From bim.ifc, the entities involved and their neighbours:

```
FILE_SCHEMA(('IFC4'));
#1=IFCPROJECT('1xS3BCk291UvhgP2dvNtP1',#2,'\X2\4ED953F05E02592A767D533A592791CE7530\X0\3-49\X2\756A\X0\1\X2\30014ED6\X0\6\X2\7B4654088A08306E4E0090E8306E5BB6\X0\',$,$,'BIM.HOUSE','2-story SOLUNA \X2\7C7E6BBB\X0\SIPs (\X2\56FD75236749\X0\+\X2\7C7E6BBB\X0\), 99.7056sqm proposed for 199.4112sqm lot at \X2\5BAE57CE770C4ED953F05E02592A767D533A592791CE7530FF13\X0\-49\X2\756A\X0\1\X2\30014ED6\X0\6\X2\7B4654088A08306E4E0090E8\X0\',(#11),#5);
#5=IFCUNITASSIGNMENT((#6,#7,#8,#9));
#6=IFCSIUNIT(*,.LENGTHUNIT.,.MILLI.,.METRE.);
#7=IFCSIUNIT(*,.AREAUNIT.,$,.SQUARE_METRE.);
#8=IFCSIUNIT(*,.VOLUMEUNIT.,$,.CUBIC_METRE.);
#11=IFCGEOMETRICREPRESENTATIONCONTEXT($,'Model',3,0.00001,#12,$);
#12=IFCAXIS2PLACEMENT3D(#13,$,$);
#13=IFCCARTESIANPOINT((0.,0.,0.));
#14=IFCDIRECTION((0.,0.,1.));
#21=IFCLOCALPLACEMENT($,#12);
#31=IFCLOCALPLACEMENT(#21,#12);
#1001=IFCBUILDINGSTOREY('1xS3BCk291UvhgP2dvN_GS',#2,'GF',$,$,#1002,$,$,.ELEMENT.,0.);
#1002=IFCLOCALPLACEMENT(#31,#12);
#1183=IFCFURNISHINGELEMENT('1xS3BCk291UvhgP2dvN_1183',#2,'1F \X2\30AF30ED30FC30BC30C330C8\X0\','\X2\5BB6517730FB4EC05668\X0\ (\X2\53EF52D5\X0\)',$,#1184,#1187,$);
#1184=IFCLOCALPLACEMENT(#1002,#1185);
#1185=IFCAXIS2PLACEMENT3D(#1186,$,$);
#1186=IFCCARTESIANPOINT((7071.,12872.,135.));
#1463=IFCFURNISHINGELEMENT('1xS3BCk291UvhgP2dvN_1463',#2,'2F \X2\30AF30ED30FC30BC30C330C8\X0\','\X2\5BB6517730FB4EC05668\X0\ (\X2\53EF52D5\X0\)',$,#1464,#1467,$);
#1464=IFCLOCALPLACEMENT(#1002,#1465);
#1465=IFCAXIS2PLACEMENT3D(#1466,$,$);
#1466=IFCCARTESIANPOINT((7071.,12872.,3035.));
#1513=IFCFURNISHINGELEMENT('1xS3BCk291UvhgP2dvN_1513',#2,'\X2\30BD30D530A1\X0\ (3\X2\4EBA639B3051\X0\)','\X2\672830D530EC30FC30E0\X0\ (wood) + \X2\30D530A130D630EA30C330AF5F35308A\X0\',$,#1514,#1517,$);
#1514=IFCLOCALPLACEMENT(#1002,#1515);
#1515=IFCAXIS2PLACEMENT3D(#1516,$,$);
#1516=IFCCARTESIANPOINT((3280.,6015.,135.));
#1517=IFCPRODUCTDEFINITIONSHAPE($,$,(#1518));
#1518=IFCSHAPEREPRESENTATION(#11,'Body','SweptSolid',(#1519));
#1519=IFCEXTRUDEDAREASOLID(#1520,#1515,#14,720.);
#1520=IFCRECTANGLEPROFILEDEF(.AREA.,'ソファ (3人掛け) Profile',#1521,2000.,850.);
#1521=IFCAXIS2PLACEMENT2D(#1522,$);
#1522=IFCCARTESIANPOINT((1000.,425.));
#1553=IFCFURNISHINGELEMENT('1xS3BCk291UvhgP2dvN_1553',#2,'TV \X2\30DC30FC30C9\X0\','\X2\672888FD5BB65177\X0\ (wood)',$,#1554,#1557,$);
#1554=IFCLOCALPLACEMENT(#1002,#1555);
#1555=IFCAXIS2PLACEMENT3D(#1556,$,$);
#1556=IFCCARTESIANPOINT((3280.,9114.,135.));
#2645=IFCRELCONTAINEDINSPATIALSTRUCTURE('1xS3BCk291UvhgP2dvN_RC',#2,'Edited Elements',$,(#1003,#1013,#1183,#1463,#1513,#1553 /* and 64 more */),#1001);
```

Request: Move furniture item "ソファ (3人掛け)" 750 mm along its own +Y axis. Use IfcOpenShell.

```python
import ifcopenshell
import ifcopenshell.api.geometry
import ifcopenshell.util.placement
import ifcopenshell.util.unit

model = ifcopenshell.open("bim.ifc")
unit_scale = ifcopenshell.util.unit.calculate_unit_scale(model)

item = model.by_guid("1xS3BCk291UvhgP2dvN_1513")
matrix = ifcopenshell.util.placement.get_local_placement(item.ObjectPlacement)
matrix[:3, 3] += matrix[:3, 1] * 0.75 / unit_scale
ifcopenshell.api.geometry.edit_object_placement(model, product=item, matrix=matrix, is_si=False)

print(ifcopenshell.util.placement.get_local_placement(item.ObjectPlacement).round(3) + 0.0)

model.write("bim_v2.ifc")
```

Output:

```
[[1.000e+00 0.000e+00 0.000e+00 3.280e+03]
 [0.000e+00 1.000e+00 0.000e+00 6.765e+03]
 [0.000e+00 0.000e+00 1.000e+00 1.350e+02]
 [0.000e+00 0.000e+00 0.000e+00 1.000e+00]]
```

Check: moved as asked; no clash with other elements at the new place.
